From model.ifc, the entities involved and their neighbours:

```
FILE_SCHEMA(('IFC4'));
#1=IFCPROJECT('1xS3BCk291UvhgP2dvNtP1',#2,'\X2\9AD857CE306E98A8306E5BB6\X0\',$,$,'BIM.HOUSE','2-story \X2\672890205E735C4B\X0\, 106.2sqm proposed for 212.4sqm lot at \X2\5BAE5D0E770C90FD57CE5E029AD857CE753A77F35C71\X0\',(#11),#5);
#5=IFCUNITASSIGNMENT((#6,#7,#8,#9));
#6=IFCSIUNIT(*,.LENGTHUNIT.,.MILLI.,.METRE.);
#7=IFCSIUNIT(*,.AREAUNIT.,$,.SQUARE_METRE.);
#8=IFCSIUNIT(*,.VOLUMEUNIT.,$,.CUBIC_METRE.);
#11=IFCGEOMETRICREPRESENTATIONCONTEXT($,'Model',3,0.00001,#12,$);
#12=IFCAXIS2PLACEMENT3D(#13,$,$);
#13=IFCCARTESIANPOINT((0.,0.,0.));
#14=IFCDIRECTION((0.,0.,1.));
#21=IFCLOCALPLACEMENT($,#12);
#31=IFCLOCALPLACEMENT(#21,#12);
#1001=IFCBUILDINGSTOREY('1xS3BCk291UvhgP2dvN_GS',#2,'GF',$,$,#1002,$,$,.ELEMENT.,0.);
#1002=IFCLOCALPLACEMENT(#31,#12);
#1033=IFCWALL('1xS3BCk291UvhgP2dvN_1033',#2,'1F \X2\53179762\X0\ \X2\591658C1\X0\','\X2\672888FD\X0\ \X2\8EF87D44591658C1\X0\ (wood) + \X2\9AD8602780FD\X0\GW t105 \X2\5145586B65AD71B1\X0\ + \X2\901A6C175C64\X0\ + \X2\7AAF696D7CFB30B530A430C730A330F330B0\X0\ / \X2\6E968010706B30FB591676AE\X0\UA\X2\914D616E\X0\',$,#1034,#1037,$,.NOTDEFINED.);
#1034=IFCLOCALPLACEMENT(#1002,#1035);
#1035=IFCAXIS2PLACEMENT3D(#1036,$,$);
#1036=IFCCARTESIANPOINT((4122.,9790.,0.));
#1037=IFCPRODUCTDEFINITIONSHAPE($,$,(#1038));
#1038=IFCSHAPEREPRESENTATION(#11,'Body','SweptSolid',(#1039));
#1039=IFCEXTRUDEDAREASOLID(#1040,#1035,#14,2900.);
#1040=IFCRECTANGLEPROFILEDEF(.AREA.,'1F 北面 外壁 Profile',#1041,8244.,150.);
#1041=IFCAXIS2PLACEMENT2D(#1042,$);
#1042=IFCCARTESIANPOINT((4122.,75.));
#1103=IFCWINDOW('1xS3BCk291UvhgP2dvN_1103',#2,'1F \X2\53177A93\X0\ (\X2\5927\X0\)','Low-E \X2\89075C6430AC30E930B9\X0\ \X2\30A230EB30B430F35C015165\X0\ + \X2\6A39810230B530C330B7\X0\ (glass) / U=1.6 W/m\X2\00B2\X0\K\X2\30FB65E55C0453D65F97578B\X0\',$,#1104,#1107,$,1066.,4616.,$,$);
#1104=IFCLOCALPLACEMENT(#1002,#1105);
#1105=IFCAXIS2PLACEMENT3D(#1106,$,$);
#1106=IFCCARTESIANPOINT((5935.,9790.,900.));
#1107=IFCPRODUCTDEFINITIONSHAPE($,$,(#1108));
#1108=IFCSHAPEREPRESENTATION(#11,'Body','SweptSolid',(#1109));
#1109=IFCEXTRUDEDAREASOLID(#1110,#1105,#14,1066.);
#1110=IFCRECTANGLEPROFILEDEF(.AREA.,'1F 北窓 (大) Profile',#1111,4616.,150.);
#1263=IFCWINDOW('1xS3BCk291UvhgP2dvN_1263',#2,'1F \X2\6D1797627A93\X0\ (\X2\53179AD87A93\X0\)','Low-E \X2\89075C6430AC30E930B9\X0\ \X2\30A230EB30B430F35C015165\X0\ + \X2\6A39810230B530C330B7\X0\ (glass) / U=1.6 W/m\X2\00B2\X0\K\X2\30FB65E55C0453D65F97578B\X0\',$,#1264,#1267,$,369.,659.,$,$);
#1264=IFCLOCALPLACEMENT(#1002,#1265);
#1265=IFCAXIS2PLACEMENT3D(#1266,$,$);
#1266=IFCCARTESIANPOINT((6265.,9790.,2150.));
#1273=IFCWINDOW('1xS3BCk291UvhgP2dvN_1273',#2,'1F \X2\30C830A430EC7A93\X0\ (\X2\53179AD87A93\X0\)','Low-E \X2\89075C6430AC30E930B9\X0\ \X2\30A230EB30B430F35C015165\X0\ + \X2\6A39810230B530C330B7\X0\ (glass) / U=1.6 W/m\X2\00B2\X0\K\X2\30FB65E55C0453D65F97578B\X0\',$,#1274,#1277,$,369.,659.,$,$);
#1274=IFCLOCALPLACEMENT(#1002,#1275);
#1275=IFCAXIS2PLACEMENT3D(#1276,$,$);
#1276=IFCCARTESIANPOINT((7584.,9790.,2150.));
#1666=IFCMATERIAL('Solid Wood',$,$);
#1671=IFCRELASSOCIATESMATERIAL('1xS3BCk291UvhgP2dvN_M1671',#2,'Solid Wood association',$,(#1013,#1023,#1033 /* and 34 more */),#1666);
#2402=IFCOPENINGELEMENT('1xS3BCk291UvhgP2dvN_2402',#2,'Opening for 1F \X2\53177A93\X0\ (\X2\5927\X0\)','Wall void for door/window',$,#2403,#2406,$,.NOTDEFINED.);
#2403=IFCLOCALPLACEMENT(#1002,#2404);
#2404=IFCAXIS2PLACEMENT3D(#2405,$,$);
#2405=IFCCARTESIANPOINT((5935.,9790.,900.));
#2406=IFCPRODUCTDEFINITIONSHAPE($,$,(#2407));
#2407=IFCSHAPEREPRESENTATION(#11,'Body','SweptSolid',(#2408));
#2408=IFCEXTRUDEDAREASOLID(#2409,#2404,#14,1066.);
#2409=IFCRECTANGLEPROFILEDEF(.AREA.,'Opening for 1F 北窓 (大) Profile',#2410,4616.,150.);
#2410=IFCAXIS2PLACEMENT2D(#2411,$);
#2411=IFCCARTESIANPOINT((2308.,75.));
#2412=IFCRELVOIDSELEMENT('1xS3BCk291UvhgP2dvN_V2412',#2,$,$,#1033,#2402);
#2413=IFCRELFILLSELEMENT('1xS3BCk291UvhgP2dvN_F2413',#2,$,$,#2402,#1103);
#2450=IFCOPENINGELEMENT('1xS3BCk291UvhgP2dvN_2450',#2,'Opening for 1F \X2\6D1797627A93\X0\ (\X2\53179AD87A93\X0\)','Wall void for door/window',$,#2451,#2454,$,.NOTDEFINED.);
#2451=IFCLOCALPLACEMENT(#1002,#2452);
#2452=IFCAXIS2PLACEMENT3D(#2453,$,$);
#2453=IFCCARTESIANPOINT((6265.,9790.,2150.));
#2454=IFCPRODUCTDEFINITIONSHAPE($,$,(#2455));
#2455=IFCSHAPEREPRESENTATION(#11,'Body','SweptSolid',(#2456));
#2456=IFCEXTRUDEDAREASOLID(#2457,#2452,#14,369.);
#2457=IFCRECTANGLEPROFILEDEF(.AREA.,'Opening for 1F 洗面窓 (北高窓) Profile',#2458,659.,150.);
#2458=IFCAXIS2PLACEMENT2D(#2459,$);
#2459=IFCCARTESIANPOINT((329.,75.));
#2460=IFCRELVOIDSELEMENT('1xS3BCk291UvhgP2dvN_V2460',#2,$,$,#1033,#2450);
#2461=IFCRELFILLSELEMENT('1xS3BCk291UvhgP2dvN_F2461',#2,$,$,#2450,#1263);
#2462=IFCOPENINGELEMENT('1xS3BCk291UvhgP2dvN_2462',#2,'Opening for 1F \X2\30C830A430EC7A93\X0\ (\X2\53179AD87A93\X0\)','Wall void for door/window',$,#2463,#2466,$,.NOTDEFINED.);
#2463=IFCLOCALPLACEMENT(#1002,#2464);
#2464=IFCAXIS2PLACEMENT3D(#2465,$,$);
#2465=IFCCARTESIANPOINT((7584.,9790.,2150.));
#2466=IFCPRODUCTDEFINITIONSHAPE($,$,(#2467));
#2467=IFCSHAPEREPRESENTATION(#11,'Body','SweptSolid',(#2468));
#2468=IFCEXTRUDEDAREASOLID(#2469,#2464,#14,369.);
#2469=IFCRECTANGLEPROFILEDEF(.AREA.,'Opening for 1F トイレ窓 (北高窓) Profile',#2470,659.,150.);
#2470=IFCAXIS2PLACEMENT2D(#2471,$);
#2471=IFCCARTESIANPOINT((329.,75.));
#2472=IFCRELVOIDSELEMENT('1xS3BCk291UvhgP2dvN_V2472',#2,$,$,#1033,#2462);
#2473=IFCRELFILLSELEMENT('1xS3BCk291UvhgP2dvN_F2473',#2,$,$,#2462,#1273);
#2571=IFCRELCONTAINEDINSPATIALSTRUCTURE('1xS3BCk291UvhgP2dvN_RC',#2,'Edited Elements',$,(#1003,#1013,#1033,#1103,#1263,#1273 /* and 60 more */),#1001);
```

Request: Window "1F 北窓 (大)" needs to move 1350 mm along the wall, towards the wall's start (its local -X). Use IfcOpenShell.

```python
import ifcopenshell
import ifcopenshell.api.geometry
import ifcopenshell.util.placement

model = ifcopenshell.open("model.ifc")

window = model.by_guid("1xS3BCk291UvhgP2dvN_1103")
opening = window.FillsVoids[0].RelatingOpeningElement
wall = opening.VoidsElements[0].RelatingBuildingElement

wall_matrix = ifcopenshell.util.placement.get_local_placement(wall.ObjectPlacement)
shift = wall_matrix[:3, 0] * -1350.0
before = ifcopenshell.util.placement.get_local_placement(window.ObjectPlacement)[:3, 3].copy()

# The window is not placed relative to its opening, so move both.
for product in (opening, window):
    matrix = ifcopenshell.util.placement.get_local_placement(product.ObjectPlacement)
    matrix[:3, 3] += shift
    ifcopenshell.api.geometry.edit_object_placement(model, product=product, matrix=matrix, is_si=False)

after = ifcopenshell.util.placement.get_local_placement(window.ObjectPlacement)[:3, 3]
print("window moved by", (after - before).round(3) + 0.0)

model.write("model_edited.ifc")
```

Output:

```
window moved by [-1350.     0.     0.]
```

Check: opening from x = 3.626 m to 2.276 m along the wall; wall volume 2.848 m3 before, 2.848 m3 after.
